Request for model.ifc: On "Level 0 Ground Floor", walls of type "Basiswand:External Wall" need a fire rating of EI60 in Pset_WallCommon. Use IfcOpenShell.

First a look at what the model holds.

```python
import ifcopenshell
import ifcopenshell.util.element

model = ifcopenshell.open("model.ifc")
print(model.schema)
storey = next(s for s in model.by_type("IfcBuildingStorey") if s.Name == "Level 0 Ground Floor")
walls = [e for e in ifcopenshell.util.element.get_decomposition(storey) if e.is_a("IfcWall")]
seen = {}
for e in walls:
    element_type = ifcopenshell.util.element.get_type(e)
    key = (element_type.Name if element_type != e and element_type else None, ifcopenshell.util.element.get_pset(e, "Pset_WallCommon", "FireRating"))
    seen[key] = seen.get(key, 0) + 1
for (name, value), count in sorted(seen.items(), key=str):
    print(count, "x", name, "|", value)
```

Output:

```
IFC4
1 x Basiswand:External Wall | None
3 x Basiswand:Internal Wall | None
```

```python
import ifcopenshell
import ifcopenshell.api.pset
import ifcopenshell.util.element

model = ifcopenshell.open("model.ifc")

storey = next(s for s in model.by_type("IfcBuildingStorey") if s.Name == "Level 0 Ground Floor")
walls = [e for e in ifcopenshell.util.element.get_decomposition(storey) if e.is_a("IfcWall")]

count = 0
for e in walls:
    element_type = ifcopenshell.util.element.get_type(e)
    if element_type in (None, e) or element_type.Name != "Basiswand:External Wall":
        continue
    # add_pset returns the element's existing set when there is one.
    pset = ifcopenshell.api.pset.add_pset(model, product=e, name="Pset_WallCommon")
    ifcopenshell.api.pset.edit_pset(model, pset=pset, properties={"FireRating": "EI60"})
    count += 1

print(count, "walls updated")

model.write("model_updated.ifc")
```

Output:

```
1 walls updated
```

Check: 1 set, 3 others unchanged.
